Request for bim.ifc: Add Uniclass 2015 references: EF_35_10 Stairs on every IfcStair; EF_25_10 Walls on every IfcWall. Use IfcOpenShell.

First a look at what the model holds.

```python
import ifcopenshell

model = ifcopenshell.open("bim.ifc")
print(model.schema)
print("classifications:", [c.Name for c in model.by_type("IfcClassification")])
for ifc_class in ("IfcDoor", "IfcRoof", "IfcStair", "IfcWall", "IfcWindow"):
    print(ifc_class, len(model.by_type(ifc_class)))
```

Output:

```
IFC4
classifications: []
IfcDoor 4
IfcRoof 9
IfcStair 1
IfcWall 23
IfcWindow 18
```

```python
import ifcopenshell
import ifcopenshell.api.classification

model = ifcopenshell.open("bim.ifc")

system = ifcopenshell.api.classification.add_classification(model, classification="Uniclass 2015")

codes = {
    "IfcStair": ("EF_35_10", "Stairs"),
    "IfcWall": ("EF_25_10", "Walls"),
}
for ifc_class, (code, name) in codes.items():
    products = model.by_type(ifc_class)
    ifcopenshell.api.classification.add_reference(
        model, products=products, classification=system, identification=code, name=name
    )
    print(code, len(products))

model.write("bim-out.ifc")
```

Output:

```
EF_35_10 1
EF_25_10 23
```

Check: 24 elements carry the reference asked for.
